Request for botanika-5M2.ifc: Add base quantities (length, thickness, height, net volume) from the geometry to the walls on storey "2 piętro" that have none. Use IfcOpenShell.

First a look at what the model holds.

```python
import ifcopenshell
import ifcopenshell.util.element
import ifcopenshell.util.unit

model = ifcopenshell.open("botanika-5M2.ifc")
print(model.schema)
for unit_type in ("LENGTHUNIT", "AREAUNIT", "VOLUMEUNIT"):
    print(unit_type, ifcopenshell.util.unit.calculate_unit_scale(model, unit_type))
storey = next(s for s in model.by_type("IfcBuildingStorey") if s.Name == "2 piętro")
walls = [e for e in ifcopenshell.util.element.get_decomposition(storey) if e.is_a("IfcWall")]
for e in sorted(walls, key=lambda e: e.id()):
    print(e.id(), e.is_a(), e.Name, list(ifcopenshell.util.element.get_psets(e, qtos_only=True)), sep=" | ")
```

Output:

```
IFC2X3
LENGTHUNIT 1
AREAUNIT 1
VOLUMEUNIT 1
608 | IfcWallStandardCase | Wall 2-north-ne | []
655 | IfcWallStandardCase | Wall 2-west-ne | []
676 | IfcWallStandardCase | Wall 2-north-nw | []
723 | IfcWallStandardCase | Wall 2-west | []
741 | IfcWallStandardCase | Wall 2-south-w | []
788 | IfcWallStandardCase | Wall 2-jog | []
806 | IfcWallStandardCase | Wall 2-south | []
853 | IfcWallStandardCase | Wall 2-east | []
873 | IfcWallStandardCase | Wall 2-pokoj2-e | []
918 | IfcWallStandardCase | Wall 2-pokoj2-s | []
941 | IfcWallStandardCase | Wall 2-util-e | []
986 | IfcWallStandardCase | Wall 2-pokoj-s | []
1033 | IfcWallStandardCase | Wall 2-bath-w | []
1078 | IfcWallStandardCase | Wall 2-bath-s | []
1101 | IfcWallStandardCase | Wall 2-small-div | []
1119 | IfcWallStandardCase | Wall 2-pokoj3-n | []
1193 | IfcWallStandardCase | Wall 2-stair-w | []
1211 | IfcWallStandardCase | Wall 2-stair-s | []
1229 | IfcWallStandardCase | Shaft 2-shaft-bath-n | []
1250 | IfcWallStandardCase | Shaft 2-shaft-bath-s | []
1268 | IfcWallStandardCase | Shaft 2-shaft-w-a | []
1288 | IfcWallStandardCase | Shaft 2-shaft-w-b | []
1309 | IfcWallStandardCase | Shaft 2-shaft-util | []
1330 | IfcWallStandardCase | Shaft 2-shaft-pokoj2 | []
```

```python
import ifcopenshell
import ifcopenshell.api.pset
import ifcopenshell.geom
import ifcopenshell.util.element
import ifcopenshell.util.shape
import ifcopenshell.util.unit

model = ifcopenshell.open("botanika-5M2.ifc")
unit_scale = ifcopenshell.util.unit.calculate_unit_scale(model)
volume_scale = ifcopenshell.util.unit.calculate_unit_scale(model, "VOLUMEUNIT")
settings = ifcopenshell.geom.settings()

storey = next(s for s in model.by_type("IfcBuildingStorey") if s.Name == "2 piętro")
walls = [e for e in ifcopenshell.util.element.get_decomposition(storey) if e.is_a("IfcWall")]

for e in sorted(walls, key=lambda e: e.id()):
    if ifcopenshell.util.element.get_psets(e, qtos_only=True, should_inherit=False):
        continue
    # Geometry comes back in metres, in the element's own axes.
    shape = ifcopenshell.geom.create_shape(settings, e)
    values = {
        "Length": ifcopenshell.util.shape.get_x(shape.geometry) / unit_scale,
        "Width": ifcopenshell.util.shape.get_y(shape.geometry) / unit_scale,
        "Height": ifcopenshell.util.shape.get_z(shape.geometry) / unit_scale,
        "NetVolume": ifcopenshell.util.shape.get_volume(shape.geometry) / volume_scale,
    }
    qto = ifcopenshell.api.pset.add_qto(model, product=e, name="BaseQuantities")
    ifcopenshell.api.pset.edit_qto(model, qto=qto, properties=values)
    print(e.id(), {k: round(v, 3) for k, v in values.items()})

model.write("botanika-5M2-out.ifc")
```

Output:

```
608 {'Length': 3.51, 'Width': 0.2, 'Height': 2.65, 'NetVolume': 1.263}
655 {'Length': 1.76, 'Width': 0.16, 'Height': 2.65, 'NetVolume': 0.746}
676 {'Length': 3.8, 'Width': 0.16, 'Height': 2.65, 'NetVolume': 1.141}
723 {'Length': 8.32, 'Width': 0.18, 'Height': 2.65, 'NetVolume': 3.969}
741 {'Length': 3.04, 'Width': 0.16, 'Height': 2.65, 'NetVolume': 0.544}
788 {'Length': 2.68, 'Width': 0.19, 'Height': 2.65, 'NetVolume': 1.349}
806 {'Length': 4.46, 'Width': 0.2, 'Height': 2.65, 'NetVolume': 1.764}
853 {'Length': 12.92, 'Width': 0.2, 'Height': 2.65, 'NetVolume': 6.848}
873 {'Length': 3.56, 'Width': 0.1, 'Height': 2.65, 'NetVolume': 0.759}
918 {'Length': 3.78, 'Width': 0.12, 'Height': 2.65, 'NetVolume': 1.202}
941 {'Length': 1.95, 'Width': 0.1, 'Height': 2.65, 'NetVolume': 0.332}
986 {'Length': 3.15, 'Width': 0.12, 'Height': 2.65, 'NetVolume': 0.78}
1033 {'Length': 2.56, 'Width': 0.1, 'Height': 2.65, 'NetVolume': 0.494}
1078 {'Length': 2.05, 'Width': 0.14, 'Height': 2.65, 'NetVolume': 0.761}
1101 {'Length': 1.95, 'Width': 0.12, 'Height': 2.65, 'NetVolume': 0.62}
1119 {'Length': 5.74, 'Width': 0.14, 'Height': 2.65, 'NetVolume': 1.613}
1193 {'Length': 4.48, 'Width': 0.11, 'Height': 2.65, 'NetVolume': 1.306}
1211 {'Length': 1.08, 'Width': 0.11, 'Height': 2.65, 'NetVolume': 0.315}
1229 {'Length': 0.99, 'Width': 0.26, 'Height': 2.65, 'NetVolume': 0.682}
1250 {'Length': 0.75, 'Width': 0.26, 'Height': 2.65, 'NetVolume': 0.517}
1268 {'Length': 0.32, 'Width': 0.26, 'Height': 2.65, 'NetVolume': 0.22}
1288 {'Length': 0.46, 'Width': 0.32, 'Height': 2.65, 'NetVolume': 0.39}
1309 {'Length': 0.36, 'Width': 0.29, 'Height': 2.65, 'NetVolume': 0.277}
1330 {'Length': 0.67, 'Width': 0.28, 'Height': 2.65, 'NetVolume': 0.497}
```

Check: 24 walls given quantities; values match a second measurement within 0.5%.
